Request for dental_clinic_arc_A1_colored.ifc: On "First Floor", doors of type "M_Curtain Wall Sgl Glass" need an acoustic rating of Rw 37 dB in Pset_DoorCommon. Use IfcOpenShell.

First a look at what the model holds.

```python
import ifcopenshell
import ifcopenshell.util.element

model = ifcopenshell.open("dental_clinic_arc_A1_colored.ifc")
print(model.schema)
storey = next(s for s in model.by_type("IfcBuildingStorey") if s.Name == "First Floor")
doors = [e for e in ifcopenshell.util.element.get_decomposition(storey) if e.is_a("IfcDoor")]
seen = {}
for e in doors:
    element_type = ifcopenshell.util.element.get_type(e)
    key = (element_type.Name if element_type != e and element_type else None, ifcopenshell.util.element.get_pset(e, "Pset_DoorCommon", "AcousticRating"))
    seen[key] = seen.get(key, 0) + 1
for (name, value), count in sorted(seen.items(), key=str):
    print(count, "x", name, "|", value)
```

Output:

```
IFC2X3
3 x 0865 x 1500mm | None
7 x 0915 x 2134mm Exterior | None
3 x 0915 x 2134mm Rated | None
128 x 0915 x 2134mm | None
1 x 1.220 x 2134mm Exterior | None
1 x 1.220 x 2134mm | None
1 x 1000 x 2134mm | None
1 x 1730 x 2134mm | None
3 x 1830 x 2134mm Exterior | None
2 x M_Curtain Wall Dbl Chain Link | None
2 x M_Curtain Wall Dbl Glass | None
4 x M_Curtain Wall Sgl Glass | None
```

```python
import ifcopenshell
import ifcopenshell.api.pset
import ifcopenshell.util.element

model = ifcopenshell.open("dental_clinic_arc_A1_colored.ifc")

storey = next(s for s in model.by_type("IfcBuildingStorey") if s.Name == "First Floor")
doors = [e for e in ifcopenshell.util.element.get_decomposition(storey) if e.is_a("IfcDoor")]

count = 0
for e in doors:
    element_type = ifcopenshell.util.element.get_type(e)
    if element_type in (None, e) or element_type.Name != "M_Curtain Wall Sgl Glass":
        continue
    # add_pset returns the element's existing set when there is one.
    pset = ifcopenshell.api.pset.add_pset(model, product=e, name="Pset_DoorCommon")
    ifcopenshell.api.pset.edit_pset(model, pset=pset, properties={"AcousticRating": "Rw 37 dB"})
    count += 1

print(count, "doors updated")

model.write("dental_clinic_arc_A1_colored_edited.ifc")
```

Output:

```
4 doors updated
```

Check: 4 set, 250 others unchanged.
